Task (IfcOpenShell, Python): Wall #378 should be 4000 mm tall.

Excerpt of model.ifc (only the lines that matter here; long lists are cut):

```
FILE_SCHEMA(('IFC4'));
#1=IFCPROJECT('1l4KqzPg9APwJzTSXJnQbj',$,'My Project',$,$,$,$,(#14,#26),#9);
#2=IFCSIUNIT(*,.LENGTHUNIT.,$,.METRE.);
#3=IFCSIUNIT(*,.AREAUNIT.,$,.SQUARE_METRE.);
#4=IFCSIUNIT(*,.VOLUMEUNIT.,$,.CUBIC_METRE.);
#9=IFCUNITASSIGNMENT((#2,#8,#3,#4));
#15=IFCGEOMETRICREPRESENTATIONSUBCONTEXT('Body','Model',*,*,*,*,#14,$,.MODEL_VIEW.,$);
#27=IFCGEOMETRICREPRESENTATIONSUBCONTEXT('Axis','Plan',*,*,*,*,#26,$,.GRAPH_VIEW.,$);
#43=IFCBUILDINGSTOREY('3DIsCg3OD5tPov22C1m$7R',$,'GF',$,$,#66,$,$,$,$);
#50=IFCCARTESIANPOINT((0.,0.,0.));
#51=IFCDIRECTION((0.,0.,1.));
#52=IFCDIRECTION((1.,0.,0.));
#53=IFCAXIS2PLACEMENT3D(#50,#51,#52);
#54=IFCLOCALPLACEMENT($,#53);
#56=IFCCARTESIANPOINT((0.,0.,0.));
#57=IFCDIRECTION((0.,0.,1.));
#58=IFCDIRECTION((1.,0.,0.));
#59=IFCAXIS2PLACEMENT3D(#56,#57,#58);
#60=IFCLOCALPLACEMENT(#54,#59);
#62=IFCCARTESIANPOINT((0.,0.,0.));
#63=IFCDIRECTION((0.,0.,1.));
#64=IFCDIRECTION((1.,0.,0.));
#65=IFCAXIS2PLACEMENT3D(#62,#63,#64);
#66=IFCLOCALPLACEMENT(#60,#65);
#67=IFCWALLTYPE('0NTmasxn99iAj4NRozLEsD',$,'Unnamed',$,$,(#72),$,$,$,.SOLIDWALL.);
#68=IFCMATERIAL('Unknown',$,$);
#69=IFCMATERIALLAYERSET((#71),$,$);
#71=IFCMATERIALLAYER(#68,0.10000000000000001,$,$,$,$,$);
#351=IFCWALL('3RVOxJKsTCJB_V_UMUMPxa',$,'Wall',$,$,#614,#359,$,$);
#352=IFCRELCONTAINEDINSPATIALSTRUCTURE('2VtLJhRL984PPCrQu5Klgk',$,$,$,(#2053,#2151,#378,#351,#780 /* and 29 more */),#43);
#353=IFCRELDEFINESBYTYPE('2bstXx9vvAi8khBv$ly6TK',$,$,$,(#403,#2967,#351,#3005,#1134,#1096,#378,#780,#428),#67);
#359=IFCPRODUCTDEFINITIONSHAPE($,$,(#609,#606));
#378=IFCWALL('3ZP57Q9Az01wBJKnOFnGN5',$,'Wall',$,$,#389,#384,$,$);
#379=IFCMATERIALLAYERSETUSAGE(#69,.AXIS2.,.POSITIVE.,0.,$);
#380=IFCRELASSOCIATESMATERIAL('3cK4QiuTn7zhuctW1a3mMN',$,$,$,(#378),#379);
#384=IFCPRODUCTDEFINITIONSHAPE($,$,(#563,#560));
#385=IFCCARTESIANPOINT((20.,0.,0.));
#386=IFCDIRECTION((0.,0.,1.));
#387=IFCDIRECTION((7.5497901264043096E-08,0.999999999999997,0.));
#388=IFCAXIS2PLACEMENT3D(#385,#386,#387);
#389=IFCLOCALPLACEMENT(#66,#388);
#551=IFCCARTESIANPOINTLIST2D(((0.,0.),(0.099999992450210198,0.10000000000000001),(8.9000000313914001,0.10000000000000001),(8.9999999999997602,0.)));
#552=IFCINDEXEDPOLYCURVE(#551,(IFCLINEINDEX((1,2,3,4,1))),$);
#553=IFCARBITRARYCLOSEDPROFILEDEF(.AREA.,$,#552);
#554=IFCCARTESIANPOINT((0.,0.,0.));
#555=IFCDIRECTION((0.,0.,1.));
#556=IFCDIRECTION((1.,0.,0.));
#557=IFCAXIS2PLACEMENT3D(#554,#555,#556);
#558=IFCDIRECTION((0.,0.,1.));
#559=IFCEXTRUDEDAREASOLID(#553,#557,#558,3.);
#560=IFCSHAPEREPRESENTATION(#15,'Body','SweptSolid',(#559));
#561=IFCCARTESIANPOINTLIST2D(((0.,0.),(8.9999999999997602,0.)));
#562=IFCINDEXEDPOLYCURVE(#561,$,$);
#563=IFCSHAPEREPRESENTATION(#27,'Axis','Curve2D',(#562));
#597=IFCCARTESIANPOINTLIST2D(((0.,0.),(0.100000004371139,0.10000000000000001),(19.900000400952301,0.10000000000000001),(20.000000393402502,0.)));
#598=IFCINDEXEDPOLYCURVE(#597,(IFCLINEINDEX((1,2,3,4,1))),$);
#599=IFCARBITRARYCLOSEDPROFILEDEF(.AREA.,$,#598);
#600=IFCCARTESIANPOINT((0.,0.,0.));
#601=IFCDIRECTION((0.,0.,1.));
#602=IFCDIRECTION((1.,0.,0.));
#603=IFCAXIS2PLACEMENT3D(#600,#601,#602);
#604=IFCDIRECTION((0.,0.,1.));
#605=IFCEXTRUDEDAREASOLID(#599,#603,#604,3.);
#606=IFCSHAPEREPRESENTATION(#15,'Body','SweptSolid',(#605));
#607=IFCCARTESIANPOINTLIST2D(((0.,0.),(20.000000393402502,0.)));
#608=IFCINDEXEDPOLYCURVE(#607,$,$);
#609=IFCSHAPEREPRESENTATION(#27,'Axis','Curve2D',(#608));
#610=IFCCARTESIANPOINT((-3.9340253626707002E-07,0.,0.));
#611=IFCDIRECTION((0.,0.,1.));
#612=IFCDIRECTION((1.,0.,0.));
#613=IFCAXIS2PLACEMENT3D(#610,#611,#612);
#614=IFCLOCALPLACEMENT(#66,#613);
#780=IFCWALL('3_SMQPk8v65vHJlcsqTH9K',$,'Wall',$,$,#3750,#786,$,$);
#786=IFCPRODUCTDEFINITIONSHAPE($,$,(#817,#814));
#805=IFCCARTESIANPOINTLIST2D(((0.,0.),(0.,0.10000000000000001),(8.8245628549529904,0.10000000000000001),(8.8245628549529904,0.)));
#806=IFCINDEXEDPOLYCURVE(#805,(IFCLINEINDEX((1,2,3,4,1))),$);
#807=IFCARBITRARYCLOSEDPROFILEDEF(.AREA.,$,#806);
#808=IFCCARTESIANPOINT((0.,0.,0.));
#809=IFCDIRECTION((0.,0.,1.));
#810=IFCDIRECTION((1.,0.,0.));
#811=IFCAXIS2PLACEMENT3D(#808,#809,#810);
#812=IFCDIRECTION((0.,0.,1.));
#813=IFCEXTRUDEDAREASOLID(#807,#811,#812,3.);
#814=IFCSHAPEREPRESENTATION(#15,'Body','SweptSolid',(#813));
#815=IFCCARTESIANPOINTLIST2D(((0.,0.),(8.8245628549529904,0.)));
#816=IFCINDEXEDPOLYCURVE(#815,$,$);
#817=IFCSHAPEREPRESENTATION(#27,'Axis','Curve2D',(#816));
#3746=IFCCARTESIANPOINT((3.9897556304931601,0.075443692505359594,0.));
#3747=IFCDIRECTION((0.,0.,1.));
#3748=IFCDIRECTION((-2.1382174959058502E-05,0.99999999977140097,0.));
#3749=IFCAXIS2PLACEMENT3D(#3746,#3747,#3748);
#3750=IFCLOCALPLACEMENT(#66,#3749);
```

```python
import ifcopenshell
import ifcopenshell.geom
import ifcopenshell.util.representation
import ifcopenshell.util.shape
import ifcopenshell.util.unit

model = ifcopenshell.open("model.ifc")
unit_scale = ifcopenshell.util.unit.calculate_unit_scale(model)
settings = ifcopenshell.geom.settings()


def volume(element):
    """Net volume in cubic metres, openings subtracted."""
    shape = ifcopenshell.geom.create_shape(settings, element)
    return ifcopenshell.util.shape.get_volume(shape.geometry)


wall = model.by_id(378)
before = volume(wall)

body = ifcopenshell.util.representation.get_representation(wall, "Model", "Body")
solid = body.Items[0]
old_height = solid.Depth
solid.Depth = 4 / unit_scale
after = volume(wall)

print(f"height {old_height:g} -> {solid.Depth:g}, volume {before:.3f} -> {after:.3f} m3")

model.write("model-out.ifc")
```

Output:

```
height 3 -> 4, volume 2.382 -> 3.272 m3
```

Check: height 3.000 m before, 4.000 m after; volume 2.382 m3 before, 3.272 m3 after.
